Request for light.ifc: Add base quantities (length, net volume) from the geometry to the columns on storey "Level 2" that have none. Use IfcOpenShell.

First a look at what the model holds.

```python
import ifcopenshell
import ifcopenshell.util.element
import ifcopenshell.util.unit

model = ifcopenshell.open("light.ifc")
print(model.schema)
for unit_type in ("LENGTHUNIT", "AREAUNIT", "VOLUMEUNIT"):
    print(unit_type, ifcopenshell.util.unit.calculate_unit_scale(model, unit_type))
storey = next(s for s in model.by_type("IfcBuildingStorey") if s.Name == "Level 2")
columns = [e for e in ifcopenshell.util.element.get_decomposition(storey) if e.is_a("IfcColumn")]
for e in sorted(columns, key=lambda e: e.id()):
    print(e.id(), e.is_a(), e.Name, list(ifcopenshell.util.element.get_psets(e, qtos_only=True)), sep=" | ")
```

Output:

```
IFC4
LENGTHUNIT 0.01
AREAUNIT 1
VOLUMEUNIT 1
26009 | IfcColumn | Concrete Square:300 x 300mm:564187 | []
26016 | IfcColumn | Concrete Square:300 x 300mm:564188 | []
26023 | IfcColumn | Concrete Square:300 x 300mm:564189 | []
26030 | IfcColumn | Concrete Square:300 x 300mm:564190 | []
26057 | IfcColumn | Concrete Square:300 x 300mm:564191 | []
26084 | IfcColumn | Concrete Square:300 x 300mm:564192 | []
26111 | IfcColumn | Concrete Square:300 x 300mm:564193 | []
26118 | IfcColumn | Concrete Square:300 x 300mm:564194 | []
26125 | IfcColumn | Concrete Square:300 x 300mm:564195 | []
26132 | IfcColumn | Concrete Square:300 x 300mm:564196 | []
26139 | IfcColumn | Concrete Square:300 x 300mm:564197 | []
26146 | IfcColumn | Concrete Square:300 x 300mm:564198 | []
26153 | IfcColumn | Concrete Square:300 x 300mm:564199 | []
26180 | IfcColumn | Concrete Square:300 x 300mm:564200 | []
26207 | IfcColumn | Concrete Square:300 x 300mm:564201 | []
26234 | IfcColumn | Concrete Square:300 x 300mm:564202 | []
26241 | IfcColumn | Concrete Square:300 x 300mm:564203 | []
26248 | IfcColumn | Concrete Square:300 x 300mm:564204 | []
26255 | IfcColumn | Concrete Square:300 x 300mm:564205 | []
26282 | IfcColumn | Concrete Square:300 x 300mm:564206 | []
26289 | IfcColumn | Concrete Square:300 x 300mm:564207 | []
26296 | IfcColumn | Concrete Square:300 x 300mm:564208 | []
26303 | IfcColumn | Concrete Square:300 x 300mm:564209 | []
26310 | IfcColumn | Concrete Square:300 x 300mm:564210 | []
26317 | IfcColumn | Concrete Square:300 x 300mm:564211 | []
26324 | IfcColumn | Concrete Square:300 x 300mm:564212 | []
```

```python
import ifcopenshell
import ifcopenshell.api.pset
import ifcopenshell.geom
import ifcopenshell.util.element
import ifcopenshell.util.shape
import ifcopenshell.util.unit

model = ifcopenshell.open("light.ifc")
unit_scale = ifcopenshell.util.unit.calculate_unit_scale(model)
volume_scale = ifcopenshell.util.unit.calculate_unit_scale(model, "VOLUMEUNIT")
settings = ifcopenshell.geom.settings()

storey = next(s for s in model.by_type("IfcBuildingStorey") if s.Name == "Level 2")
columns = [e for e in ifcopenshell.util.element.get_decomposition(storey) if e.is_a("IfcColumn")]

for e in sorted(columns, key=lambda e: e.id()):
    if ifcopenshell.util.element.get_psets(e, qtos_only=True, should_inherit=False):
        continue
    # Geometry comes back in metres, in the element's own axes.
    shape = ifcopenshell.geom.create_shape(settings, e)
    values = {
        "Length": ifcopenshell.util.shape.get_z(shape.geometry) / unit_scale,
        "NetVolume": ifcopenshell.util.shape.get_volume(shape.geometry) / volume_scale,
    }
    qto = ifcopenshell.api.pset.add_qto(model, product=e, name="Qto_ColumnBaseQuantities")
    ifcopenshell.api.pset.edit_qto(model, qto=qto, properties=values)
    print(e.id(), {k: round(v, 3) for k, v in values.items()})

model.write("light-out.ifc")
```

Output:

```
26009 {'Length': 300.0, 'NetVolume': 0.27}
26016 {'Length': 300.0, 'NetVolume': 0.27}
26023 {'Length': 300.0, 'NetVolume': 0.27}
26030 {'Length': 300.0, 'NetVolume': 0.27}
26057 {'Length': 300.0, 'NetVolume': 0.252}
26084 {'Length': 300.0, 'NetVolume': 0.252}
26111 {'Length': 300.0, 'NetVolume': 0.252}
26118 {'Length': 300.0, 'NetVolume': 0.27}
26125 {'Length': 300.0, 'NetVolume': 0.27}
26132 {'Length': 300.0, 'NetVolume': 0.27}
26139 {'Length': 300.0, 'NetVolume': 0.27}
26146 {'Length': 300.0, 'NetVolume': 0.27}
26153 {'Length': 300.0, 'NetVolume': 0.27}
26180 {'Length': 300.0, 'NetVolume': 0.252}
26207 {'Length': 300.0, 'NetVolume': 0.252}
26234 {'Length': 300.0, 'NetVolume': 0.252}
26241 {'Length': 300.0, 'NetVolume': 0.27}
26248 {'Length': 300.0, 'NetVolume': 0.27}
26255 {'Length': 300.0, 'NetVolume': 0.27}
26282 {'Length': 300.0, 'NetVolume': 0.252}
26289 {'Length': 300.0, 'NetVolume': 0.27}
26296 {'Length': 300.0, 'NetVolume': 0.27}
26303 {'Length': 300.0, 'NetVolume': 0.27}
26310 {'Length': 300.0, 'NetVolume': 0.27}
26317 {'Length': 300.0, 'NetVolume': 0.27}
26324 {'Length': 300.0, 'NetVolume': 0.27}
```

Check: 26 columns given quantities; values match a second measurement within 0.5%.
